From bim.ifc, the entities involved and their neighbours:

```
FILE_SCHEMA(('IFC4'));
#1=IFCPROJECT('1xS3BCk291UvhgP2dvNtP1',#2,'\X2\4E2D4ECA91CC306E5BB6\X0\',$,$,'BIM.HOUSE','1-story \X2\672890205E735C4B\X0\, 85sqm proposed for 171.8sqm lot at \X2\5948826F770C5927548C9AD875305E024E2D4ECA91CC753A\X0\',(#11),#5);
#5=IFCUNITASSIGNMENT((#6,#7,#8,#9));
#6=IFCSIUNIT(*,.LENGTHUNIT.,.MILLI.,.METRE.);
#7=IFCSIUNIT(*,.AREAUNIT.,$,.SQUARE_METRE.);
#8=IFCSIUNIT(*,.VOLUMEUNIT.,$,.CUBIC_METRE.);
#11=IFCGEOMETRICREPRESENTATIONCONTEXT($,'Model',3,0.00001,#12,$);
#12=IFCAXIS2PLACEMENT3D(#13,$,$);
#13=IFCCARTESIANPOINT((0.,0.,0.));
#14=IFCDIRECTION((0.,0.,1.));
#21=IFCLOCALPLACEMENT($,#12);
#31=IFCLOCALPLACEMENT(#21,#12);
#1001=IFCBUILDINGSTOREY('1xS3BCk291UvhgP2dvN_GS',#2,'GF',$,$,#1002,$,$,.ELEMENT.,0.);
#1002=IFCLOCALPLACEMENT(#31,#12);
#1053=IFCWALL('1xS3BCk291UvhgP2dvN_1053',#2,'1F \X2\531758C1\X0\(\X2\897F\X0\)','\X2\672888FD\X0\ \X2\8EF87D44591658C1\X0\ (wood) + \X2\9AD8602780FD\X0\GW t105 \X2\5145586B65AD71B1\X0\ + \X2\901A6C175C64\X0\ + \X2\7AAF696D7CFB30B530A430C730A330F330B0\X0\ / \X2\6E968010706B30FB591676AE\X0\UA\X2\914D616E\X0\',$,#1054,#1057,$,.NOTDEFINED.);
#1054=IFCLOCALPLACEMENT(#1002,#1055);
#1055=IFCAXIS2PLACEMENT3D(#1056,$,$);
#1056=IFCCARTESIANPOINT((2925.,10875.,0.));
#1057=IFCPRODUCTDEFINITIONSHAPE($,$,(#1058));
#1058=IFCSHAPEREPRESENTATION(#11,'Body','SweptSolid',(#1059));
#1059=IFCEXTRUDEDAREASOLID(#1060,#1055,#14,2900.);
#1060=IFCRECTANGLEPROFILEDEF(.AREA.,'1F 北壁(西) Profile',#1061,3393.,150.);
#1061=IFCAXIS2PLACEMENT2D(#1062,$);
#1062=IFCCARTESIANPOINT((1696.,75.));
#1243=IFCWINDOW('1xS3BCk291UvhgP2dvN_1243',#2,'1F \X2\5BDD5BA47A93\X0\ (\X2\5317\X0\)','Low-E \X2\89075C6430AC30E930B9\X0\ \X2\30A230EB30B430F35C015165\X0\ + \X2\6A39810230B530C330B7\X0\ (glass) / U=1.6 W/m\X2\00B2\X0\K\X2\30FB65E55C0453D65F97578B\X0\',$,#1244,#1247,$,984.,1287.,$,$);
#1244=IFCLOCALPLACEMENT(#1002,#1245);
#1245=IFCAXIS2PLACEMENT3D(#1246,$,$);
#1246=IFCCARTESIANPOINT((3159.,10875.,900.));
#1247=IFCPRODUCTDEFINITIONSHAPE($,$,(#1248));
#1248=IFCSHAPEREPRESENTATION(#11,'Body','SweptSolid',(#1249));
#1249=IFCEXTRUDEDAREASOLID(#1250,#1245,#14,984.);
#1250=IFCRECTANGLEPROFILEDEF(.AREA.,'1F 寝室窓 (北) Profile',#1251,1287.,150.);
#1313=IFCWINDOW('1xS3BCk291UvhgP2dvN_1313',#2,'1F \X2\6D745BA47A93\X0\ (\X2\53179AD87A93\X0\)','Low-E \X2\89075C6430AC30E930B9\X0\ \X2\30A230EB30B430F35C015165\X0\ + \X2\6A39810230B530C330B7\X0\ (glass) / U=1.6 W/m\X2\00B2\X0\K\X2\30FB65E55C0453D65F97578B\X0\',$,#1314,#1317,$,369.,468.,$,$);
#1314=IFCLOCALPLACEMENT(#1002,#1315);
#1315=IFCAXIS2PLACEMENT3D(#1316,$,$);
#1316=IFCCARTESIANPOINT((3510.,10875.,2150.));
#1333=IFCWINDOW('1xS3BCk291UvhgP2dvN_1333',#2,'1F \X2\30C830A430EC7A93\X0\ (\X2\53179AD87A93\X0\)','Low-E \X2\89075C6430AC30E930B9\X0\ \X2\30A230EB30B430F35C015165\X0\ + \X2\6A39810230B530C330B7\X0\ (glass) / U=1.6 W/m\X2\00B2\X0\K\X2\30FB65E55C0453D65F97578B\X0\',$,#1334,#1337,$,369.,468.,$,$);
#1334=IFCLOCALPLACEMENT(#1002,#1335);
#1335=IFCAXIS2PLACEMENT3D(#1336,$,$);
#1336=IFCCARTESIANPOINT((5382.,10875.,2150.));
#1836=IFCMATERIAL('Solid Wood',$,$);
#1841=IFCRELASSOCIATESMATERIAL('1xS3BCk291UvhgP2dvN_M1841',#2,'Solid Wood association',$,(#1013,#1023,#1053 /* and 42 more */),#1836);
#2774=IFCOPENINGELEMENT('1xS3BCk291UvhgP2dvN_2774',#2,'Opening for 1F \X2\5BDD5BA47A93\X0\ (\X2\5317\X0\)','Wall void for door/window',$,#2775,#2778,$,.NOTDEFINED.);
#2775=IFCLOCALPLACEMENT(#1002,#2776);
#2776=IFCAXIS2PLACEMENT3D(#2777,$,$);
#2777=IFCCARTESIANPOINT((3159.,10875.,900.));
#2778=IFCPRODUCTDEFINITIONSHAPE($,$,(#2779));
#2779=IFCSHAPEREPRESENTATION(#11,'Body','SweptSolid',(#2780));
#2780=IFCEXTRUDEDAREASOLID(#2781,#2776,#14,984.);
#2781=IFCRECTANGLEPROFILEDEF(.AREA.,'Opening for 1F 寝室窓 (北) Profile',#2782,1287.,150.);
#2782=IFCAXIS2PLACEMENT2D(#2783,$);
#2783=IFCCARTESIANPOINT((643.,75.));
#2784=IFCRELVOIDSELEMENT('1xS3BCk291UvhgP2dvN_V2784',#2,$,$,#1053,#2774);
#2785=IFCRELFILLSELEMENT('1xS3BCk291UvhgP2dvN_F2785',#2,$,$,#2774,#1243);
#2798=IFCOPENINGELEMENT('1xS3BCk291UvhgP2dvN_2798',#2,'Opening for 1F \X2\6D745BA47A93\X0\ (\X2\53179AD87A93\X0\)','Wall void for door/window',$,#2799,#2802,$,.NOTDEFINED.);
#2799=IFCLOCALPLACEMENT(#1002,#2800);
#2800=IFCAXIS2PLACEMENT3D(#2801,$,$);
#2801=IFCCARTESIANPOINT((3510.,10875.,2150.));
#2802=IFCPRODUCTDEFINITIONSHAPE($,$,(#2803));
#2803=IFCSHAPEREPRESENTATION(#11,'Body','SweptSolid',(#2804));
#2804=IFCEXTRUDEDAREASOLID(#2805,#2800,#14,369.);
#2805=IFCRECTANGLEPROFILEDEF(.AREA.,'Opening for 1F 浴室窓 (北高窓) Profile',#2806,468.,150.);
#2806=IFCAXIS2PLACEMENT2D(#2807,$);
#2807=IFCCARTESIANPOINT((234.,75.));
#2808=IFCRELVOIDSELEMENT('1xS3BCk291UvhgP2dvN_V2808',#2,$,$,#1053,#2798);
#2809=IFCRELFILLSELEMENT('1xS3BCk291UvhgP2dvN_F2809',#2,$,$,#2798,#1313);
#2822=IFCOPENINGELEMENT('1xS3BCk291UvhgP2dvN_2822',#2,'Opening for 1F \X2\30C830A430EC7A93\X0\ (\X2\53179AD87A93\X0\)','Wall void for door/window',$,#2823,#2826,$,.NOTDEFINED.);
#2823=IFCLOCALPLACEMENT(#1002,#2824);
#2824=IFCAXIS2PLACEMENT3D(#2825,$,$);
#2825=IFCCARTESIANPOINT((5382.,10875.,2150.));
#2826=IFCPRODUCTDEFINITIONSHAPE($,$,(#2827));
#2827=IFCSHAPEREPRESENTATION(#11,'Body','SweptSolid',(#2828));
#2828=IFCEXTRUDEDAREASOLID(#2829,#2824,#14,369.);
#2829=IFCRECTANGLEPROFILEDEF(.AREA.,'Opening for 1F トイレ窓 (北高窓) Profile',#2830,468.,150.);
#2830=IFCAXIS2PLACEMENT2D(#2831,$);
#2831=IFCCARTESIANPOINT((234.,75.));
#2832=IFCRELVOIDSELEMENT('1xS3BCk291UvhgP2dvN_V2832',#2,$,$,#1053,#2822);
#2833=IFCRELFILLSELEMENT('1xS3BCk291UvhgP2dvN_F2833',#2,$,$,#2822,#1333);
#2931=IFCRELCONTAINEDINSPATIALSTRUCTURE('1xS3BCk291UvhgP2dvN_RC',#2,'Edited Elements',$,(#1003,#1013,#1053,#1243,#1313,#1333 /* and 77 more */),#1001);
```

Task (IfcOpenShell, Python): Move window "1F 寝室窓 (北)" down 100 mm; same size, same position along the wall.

```python
import numpy as np
import ifcopenshell
import ifcopenshell.api.geometry
import ifcopenshell.util.placement
import ifcopenshell.util.unit

model = ifcopenshell.open("bim.ifc")
unit_scale = ifcopenshell.util.unit.calculate_unit_scale(model)

window = model.by_id(1243)
opening = window.FillsVoids[0].RelatingOpeningElement
dz = -100.0

shift = np.array([0.0, 0.0, dz])
# The window is not placed relative to its opening, so move both.
for product in (opening, window):
    matrix = ifcopenshell.util.placement.get_local_placement(product.ObjectPlacement)
    matrix[:3, 3] += shift
    ifcopenshell.api.geometry.edit_object_placement(model, product=product, matrix=matrix, is_si=False)

print(f"moved by {dz * unit_scale:+.3f} m")

model.write("bim-out.ifc")
```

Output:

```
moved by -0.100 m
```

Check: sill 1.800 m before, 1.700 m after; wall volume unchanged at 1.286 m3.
